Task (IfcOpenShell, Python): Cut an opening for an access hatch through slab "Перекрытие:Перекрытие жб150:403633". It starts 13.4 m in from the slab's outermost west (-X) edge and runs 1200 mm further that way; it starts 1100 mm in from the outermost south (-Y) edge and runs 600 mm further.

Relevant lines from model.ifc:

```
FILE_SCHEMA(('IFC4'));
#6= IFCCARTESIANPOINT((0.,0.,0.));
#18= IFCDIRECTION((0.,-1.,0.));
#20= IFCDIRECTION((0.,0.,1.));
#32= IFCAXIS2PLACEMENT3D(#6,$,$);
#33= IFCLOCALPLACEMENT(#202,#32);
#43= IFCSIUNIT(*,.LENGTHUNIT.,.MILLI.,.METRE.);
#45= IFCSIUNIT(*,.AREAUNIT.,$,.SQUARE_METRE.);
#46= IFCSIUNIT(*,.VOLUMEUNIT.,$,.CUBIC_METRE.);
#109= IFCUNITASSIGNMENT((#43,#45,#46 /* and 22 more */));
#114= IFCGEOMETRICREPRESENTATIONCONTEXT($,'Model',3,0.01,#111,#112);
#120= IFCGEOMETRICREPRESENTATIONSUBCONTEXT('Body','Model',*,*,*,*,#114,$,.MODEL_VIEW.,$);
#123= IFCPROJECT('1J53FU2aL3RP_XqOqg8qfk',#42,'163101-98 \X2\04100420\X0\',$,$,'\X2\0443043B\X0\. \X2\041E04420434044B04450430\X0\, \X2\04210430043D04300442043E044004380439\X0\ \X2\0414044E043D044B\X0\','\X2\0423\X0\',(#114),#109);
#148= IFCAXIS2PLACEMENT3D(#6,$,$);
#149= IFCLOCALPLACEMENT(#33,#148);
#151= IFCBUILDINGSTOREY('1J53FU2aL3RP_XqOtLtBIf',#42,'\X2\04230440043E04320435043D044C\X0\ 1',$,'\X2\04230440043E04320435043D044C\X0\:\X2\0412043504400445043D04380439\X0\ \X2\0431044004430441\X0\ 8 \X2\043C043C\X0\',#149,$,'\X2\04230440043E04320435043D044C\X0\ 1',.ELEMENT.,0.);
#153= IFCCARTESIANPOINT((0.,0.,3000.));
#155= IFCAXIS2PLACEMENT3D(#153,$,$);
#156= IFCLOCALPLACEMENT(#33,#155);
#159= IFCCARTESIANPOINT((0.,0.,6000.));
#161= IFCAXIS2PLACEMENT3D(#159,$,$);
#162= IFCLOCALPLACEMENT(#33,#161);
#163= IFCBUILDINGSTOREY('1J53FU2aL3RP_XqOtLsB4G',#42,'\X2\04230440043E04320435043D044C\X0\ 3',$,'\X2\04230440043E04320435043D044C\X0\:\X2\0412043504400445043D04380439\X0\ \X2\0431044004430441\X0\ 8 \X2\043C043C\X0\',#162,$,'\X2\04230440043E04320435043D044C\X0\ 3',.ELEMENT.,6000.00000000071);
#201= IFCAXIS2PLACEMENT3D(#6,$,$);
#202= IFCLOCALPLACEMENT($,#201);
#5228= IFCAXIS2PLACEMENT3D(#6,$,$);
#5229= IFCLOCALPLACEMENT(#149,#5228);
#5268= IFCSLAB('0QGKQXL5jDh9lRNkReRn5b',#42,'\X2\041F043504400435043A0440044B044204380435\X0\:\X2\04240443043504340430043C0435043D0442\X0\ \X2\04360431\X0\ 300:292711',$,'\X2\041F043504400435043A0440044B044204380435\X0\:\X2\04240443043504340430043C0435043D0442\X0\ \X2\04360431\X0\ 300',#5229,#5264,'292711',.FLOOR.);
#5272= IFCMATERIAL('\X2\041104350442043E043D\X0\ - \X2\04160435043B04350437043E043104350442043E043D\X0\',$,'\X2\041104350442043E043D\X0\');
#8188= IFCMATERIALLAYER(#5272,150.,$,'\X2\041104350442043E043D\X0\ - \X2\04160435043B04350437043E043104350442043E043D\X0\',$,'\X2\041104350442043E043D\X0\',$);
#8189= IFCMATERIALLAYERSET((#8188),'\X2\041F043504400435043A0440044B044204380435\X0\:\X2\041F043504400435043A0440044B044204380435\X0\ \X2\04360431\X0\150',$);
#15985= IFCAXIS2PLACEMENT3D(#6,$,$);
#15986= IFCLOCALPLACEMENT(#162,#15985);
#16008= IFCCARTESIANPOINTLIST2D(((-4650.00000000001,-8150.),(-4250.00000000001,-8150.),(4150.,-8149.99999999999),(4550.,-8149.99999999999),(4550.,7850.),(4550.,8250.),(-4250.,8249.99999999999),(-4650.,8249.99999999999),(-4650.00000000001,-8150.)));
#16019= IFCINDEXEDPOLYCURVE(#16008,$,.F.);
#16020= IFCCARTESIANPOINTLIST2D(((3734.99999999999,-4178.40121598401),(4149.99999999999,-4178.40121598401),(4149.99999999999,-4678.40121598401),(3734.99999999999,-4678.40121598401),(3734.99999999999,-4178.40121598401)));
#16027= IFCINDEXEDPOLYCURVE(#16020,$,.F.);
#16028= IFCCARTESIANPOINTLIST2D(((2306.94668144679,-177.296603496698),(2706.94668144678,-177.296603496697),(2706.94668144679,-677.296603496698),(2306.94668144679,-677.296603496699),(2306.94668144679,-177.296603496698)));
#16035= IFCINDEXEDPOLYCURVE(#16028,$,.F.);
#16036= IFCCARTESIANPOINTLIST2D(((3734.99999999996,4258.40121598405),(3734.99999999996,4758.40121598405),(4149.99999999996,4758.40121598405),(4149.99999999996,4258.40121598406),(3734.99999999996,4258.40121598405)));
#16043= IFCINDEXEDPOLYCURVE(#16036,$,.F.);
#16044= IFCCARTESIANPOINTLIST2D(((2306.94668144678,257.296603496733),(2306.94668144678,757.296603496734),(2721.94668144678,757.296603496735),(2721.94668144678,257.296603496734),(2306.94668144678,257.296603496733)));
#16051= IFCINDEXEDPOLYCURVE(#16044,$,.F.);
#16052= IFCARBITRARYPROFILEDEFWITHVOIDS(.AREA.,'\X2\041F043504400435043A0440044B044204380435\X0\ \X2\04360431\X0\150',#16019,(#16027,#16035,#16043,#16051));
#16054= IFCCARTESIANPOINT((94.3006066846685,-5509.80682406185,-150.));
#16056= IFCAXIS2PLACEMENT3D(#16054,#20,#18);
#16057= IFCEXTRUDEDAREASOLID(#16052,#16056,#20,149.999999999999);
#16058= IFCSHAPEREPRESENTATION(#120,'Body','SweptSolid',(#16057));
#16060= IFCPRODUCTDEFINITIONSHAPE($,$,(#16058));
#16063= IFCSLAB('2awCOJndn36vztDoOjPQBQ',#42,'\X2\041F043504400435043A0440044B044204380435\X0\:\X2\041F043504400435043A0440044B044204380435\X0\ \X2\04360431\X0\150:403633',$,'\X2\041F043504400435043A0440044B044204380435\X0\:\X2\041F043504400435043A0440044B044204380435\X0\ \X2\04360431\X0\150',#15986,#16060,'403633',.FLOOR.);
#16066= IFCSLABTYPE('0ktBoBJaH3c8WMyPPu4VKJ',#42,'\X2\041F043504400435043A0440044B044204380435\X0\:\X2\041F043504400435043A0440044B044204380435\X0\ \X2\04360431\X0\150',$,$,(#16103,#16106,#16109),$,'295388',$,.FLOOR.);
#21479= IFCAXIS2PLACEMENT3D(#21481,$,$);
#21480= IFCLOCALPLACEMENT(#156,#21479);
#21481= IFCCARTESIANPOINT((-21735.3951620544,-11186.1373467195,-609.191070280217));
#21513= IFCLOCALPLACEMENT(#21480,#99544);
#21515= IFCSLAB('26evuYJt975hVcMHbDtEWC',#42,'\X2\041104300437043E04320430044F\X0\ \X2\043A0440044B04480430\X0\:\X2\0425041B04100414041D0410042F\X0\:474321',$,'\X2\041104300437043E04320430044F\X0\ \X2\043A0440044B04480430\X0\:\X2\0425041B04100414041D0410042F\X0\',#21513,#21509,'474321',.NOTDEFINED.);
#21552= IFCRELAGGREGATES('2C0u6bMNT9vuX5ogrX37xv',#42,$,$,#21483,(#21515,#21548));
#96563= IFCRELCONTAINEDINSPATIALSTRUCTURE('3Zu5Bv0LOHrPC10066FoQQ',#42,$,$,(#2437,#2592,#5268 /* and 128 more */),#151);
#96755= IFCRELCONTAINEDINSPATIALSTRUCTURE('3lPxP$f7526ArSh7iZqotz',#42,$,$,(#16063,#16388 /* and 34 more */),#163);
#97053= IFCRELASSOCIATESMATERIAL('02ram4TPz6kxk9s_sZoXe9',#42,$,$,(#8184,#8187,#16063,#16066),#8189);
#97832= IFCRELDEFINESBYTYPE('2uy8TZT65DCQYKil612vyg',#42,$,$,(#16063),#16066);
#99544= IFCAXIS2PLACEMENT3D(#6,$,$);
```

```python
import numpy as np
import ifcopenshell
import ifcopenshell.api.feature
import ifcopenshell.api.geometry
import ifcopenshell.api.root
import ifcopenshell.geom
import ifcopenshell.util.placement
import ifcopenshell.util.representation
import ifcopenshell.util.shape
import ifcopenshell.util.unit

model = ifcopenshell.open("model.ifc")
unit_scale = ifcopenshell.util.unit.calculate_unit_scale(model)
settings = ifcopenshell.geom.settings()


def volume(element):
    """Net volume in cubic metres, openings subtracted."""
    shape = ifcopenshell.geom.create_shape(settings, element)
    return ifcopenshell.util.shape.get_volume(shape.geometry)


slab = model.by_guid("2awCOJndn36vztDoOjPQBQ")
before = volume(slab)

# Extent in the slab's own axes, in metres. The edges named are its -X and -Y sides.
slab_shape = ifcopenshell.geom.create_shape(settings, slab)
vertices = ifcopenshell.util.shape.get_vertices(slab_shape.geometry)
x_min, y_min, bottom = vertices.min(axis=0)
top = vertices[:, 2].max()

opening = ifcopenshell.api.root.create_entity(model, ifc_class="IfcOpeningElement", name="Access hatch opening", predefined_type="OPENING")
context = ifcopenshell.util.representation.get_context(model, "Model", "Body", "MODEL_VIEW")
width, depth = 1.2, 0.6
outline = [(0.0, 0.0), (width, 0.0), (width, depth), (0.0, depth), (0.0, 0.0)]
# Overshoot both faces by 50 mm so the cut is clean.
shape = ifcopenshell.api.geometry.add_slab_representation(
    model, context=context, depth=top - bottom + 0.1, polyline=outline
)
ifcopenshell.api.geometry.assign_representation(model, product=opening, representation=shape)

matrix = ifcopenshell.util.placement.get_local_placement(slab.ObjectPlacement)
matrix[:, 3] = matrix @ np.append(np.array([x_min + 13.4, y_min + 1.1, bottom - 0.05]) / unit_scale, 1.0)
ifcopenshell.api.geometry.edit_object_placement(model, product=opening, matrix=matrix, is_si=False)
ifcopenshell.api.feature.add_feature(model, feature=opening, element=slab)

after = volume(slab)

print(f"slab volume {before:.3f} -> {after:.3f} m3")

model.write("model_rev.ifc")
```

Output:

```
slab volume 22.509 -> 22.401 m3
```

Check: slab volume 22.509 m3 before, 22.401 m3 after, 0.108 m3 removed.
